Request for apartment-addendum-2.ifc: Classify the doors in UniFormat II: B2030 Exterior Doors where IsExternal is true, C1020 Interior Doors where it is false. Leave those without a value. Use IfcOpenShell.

First a look at what the model holds.

```python
import ifcopenshell
import ifcopenshell.util.element

model = ifcopenshell.open("apartment-addendum-2.ifc")
print(model.schema)
print("classifications:", [c.Name for c in model.by_type("IfcClassification")])
values = [ifcopenshell.util.element.get_pset(e, "Pset_DoorCommon", "IsExternal") for e in model.by_type("IfcDoor")]
for value in (True, False, None):
    print("IsExternal", value, values.count(value))
```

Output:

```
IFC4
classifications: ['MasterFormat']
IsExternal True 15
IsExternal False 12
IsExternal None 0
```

```python
import ifcopenshell
import ifcopenshell.api.classification
import ifcopenshell.util.element

model = ifcopenshell.open("apartment-addendum-2.ifc")

system = ifcopenshell.api.classification.add_classification(model, classification="UniFormat II")

doors = model.by_type("IfcDoor")
external = {e: ifcopenshell.util.element.get_pset(e, "Pset_DoorCommon", "IsExternal") for e in doors}
for flag, code, name in ((True, "B2030", "Exterior Doors"), (False, "C1020", "Interior Doors")):
    products = [e for e in doors if external[e] is flag]
    ifcopenshell.api.classification.add_reference(
        model, products=products, classification=system, identification=code, name=name
    )
    print(code, len(products))

model.write("apartment-addendum-2-out.ifc")
```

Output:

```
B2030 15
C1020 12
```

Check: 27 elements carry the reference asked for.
